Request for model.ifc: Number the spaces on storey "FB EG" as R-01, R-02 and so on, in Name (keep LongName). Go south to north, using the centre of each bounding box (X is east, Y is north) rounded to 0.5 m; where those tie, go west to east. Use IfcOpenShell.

First a look at what the model holds.

```python
import ifcopenshell
import ifcopenshell.util.element
import ifcopenshell.util.placement

model = ifcopenshell.open("model.ifc")
print(model.schema)
storey = next(s for s in model.by_type("IfcBuildingStorey") if s.Name == "FB EG")
spaces = [e for e in ifcopenshell.util.element.get_decomposition(storey) if e.is_a("IfcSpace")]
for e in sorted(spaces, key=lambda e: e.id()):
    origin = ifcopenshell.util.placement.get_local_placement(e.ObjectPlacement)[:3, 3]
    print(e.id(), e.Name, e.LongName, origin.round(2) + 0.0, sep=" | ")
```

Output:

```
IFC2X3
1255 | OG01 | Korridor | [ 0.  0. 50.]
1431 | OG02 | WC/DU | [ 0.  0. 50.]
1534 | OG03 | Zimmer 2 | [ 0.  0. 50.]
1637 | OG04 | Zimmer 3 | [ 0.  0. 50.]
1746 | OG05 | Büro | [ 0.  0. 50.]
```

```python
import ifcopenshell
import ifcopenshell.geom
import ifcopenshell.util.element
import ifcopenshell.util.shape

model = ifcopenshell.open("model.ifc")
settings = ifcopenshell.geom.settings()
settings.set("use-world-coords", True)


def centre(element):
    shape = ifcopenshell.geom.create_shape(settings, element)
    return ifcopenshell.util.shape.get_bbox_centroid(shape.geometry)


storey = next(s for s in model.by_type("IfcBuildingStorey") if s.Name == "FB EG")
spaces = [e for e in ifcopenshell.util.element.get_decomposition(storey) if e.is_a("IfcSpace")]

# Insertion points can sit at a corner or the storey origin, so sort by the geometry (in metres).
centres = {e: centre(e) for e in spaces}
spaces.sort(key=lambda e: (round(centres[e][1] / 0.5), centres[e][0]))

for i, e in enumerate(spaces, start=1):
    number = f"R-{i:02d}"
    e.Name = number
    print(e.id(), number)

model.write("model_edited.ifc")
```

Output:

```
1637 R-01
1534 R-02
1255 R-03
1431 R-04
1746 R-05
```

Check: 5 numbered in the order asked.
